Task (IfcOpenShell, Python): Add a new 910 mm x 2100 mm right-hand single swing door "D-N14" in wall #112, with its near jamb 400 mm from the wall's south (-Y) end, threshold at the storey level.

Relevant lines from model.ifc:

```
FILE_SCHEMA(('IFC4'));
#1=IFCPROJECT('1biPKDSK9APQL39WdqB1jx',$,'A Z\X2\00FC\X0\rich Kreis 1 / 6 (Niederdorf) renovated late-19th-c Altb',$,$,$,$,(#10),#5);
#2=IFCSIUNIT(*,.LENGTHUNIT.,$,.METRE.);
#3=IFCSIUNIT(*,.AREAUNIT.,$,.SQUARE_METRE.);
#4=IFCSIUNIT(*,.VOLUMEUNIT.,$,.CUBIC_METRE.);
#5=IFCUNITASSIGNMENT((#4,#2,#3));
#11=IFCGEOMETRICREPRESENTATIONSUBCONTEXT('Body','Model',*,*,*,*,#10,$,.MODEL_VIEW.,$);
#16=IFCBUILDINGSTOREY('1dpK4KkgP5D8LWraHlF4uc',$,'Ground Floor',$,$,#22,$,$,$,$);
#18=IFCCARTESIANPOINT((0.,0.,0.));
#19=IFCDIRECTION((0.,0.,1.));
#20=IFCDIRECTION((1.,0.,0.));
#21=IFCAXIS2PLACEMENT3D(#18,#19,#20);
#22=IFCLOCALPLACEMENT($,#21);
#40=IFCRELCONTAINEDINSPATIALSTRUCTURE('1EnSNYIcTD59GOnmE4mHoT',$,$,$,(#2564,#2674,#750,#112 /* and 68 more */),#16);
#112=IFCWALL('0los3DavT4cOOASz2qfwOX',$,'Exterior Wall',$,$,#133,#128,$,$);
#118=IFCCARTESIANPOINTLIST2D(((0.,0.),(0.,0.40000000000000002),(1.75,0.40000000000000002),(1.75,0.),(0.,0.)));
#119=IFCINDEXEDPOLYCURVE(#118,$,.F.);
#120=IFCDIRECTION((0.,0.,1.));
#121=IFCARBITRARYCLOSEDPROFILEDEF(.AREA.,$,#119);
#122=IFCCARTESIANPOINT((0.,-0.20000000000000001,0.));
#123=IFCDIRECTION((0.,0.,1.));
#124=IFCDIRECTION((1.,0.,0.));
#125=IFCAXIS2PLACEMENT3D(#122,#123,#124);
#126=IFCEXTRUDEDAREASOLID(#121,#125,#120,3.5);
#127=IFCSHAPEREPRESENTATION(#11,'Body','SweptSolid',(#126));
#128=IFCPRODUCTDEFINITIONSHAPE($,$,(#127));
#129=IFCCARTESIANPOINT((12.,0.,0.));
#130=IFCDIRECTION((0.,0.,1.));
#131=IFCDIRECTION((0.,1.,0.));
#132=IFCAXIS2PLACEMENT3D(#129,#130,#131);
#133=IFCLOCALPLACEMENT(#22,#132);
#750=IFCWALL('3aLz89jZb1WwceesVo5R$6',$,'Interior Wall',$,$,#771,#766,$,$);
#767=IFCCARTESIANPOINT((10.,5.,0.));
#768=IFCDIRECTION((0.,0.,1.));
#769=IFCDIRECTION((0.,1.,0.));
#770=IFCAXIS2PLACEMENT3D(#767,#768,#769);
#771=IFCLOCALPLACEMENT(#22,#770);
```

```python
import numpy as np
import ifcopenshell
import ifcopenshell.api.feature
import ifcopenshell.api.geometry
import ifcopenshell.api.root
import ifcopenshell.api.spatial
import ifcopenshell.geom
import ifcopenshell.util.element
import ifcopenshell.util.placement
import ifcopenshell.util.representation
import ifcopenshell.util.shape
import ifcopenshell.util.unit

model = ifcopenshell.open("model.ifc")
unit_scale = ifcopenshell.util.unit.calculate_unit_scale(model)
settings = ifcopenshell.geom.settings()


def volume(element):
    """Net volume in cubic metres, openings subtracted."""
    shape = ifcopenshell.geom.create_shape(settings, element)
    return ifcopenshell.util.shape.get_volume(shape.geometry)


wall = model.by_id(112)
storey = ifcopenshell.util.element.get_container(wall, ifc_class="IfcBuildingStorey")
context = ifcopenshell.util.representation.get_context(model, "Model", "Body", "MODEL_VIEW")
before = volume(wall)

width, height, from_end, sill = 0.91, 2.1, 0.4, 0.0  # metres

# The wall runs along its own X axis, and the end named is its -X end.
wall_shape = ifcopenshell.geom.create_shape(settings, wall)
x, y, z = ifcopenshell.util.shape.get_vertices(wall_shape.geometry).T
start = x.min() + from_end
face, thickness = float(y.min()), float(y.max() - y.min())
wall_matrix = ifcopenshell.util.placement.get_local_placement(wall.ObjectPlacement)
level = ifcopenshell.util.placement.get_local_placement(storey.ObjectPlacement)[2, 3]


def in_wall(x, y):
    """Placement at x, y metres in the wall's axes, at sill height."""
    matrix = wall_matrix.copy()
    matrix[:, 3] = wall_matrix @ np.array([x / unit_scale, y / unit_scale, 0.0, 1.0])
    matrix[2, 3] = level + sill / unit_scale
    return matrix


# Opening: a box that overshoots both wall faces by 50 mm.
opening = ifcopenshell.api.root.create_entity(model, ifc_class="IfcOpeningElement", predefined_type="OPENING")
box = ifcopenshell.api.geometry.add_wall_representation(
    model, context=context, length=width, height=height, thickness=thickness + 0.1
)
ifcopenshell.api.geometry.assign_representation(model, product=opening, representation=box)
ifcopenshell.api.geometry.edit_object_placement(model, product=opening, matrix=in_wall(start, face - 0.05), is_si=False)
ifcopenshell.api.feature.add_feature(model, feature=opening, element=wall)

door = ifcopenshell.api.root.create_entity(model, ifc_class="IfcDoor", name="D-N14", predefined_type="DOOR")
door.OverallWidth, door.OverallHeight = width / unit_scale, height / unit_scale
door.OperationType = "SINGLE_SWING_RIGHT"
body = ifcopenshell.api.geometry.add_door_representation(
    model,
    context=context,
    overall_width=door.OverallWidth,
    overall_height=door.OverallHeight,
    operation_type="SINGLE_SWING_RIGHT",
    lining_properties={"LiningDepth": thickness / unit_scale, "ThresholdDepth": thickness / unit_scale},
)
ifcopenshell.api.geometry.assign_representation(model, product=door, representation=body)
ifcopenshell.api.spatial.assign_container(model, products=[door], relating_structure=storey)
ifcopenshell.api.feature.add_filling(model, opening=opening, element=door)

# The lining spans the wall, so the door starts at the wall face.
ifcopenshell.api.geometry.edit_object_placement(model, product=door, matrix=in_wall(start, face), is_si=False)

after = volume(wall)

print(f"wall volume {before:.3f} -> {after:.3f} m3")

model.write("model_v2.ifc")
```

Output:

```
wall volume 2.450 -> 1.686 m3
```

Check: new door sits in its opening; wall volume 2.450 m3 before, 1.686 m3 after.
